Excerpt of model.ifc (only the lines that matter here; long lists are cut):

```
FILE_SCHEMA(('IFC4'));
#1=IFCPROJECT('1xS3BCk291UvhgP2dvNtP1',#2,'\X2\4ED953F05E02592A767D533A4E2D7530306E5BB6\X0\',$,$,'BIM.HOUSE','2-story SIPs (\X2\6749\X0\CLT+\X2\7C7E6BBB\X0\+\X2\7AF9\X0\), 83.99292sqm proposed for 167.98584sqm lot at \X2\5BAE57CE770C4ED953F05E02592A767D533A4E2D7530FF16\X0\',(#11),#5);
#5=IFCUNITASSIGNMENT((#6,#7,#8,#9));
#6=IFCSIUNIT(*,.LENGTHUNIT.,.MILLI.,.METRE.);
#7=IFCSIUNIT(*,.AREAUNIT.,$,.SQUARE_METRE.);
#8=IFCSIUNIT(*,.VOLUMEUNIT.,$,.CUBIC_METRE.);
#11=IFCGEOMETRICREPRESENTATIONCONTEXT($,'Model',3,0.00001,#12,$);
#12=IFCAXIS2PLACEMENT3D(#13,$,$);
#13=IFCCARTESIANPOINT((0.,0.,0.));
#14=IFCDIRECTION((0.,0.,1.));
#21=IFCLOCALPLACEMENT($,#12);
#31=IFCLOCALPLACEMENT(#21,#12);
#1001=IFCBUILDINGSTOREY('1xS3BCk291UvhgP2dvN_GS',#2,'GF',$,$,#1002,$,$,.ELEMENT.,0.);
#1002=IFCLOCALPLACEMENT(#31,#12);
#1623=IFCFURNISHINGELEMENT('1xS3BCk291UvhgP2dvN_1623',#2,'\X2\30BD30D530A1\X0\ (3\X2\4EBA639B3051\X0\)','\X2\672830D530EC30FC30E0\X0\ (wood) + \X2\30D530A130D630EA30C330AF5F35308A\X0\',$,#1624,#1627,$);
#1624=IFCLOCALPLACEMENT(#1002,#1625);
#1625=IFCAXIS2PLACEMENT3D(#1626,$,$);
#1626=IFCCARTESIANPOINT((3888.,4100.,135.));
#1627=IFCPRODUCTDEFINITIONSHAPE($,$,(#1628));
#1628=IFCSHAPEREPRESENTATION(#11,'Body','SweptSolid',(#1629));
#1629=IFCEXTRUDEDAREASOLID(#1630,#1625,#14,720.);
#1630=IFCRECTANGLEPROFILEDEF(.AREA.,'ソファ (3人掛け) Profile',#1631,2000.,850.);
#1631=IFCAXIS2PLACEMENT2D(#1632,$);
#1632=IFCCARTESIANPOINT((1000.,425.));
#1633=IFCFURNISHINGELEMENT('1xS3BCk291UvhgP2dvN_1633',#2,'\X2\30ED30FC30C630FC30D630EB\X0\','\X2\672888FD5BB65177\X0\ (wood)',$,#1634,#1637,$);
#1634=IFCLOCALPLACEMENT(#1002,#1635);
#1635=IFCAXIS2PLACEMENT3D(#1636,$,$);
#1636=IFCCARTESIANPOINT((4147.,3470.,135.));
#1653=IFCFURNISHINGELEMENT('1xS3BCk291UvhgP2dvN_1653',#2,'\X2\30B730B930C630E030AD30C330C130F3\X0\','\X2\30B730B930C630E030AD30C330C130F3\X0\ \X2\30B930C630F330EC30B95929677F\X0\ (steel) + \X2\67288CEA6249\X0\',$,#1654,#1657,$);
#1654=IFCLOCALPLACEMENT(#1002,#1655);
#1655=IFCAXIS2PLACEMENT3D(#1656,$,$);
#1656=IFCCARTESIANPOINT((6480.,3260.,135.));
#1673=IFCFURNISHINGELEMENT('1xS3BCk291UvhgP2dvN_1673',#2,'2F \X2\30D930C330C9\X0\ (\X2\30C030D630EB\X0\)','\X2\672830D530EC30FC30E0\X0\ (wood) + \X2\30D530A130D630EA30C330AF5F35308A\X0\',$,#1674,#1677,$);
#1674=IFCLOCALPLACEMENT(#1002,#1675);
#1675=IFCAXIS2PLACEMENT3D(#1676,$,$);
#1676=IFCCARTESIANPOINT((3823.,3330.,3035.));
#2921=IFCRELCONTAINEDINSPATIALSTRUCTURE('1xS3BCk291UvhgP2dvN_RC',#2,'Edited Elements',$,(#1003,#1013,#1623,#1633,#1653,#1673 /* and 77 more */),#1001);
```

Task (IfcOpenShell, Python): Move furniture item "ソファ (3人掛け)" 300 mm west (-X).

```python
import ifcopenshell
import ifcopenshell.api.geometry
import ifcopenshell.util.placement

model = ifcopenshell.open("model.ifc")

item = model.by_guid("1xS3BCk291UvhgP2dvN_1623")
matrix = ifcopenshell.util.placement.get_local_placement(item.ObjectPlacement)
matrix[0, 3] -= 300.0
ifcopenshell.api.geometry.edit_object_placement(model, product=item, matrix=matrix, is_si=False)

print(ifcopenshell.util.placement.get_local_placement(item.ObjectPlacement).round(3) + 0.0)

model.write("model_v2.ifc")
```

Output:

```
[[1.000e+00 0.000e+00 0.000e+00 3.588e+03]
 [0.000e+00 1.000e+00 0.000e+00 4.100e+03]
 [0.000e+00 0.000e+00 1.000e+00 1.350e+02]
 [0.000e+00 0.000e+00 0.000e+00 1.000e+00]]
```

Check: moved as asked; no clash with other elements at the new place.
